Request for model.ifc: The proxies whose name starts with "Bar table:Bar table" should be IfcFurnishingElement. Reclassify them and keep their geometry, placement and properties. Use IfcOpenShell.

First a look at what the model holds.

```python
import re

import ifcopenshell

model = ifcopenshell.open("model.ifc")
print(model.schema)
seen = {}
for e in model.by_type("IfcBuildingElementProxy"):
    name = re.sub(r":\d+(:\d+)?$", "", e.Name or "")  # drop the element id that some exporters append
    seen[name] = seen.get(name, 0) + 1
for name, count in sorted(seen.items()):
    print(count, "x", name)
```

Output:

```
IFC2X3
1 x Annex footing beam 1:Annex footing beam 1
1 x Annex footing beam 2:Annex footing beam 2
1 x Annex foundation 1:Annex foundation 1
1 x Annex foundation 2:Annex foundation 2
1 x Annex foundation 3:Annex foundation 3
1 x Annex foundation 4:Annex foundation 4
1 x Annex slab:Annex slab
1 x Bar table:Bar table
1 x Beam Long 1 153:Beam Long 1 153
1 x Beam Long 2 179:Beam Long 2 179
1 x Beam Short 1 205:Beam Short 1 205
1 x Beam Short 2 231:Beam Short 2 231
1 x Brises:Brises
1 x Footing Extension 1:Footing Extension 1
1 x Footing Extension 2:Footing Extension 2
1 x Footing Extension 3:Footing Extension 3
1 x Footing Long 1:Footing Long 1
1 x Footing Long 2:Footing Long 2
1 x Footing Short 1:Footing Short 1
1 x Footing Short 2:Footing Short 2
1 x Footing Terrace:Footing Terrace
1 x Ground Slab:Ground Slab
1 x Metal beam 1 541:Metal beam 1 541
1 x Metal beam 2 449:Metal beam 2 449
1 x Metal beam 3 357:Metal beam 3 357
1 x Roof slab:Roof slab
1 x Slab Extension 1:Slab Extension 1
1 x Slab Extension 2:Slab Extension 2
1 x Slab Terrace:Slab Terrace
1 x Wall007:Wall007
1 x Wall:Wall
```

```python
import ifcopenshell
import ifcopenshell.api.root

model = ifcopenshell.open("model.ifc")

proxies = [e.id() for e in model.by_type("IfcBuildingElementProxy") if (e.Name or "").startswith("Bar table:Bar table")]
for step_id in proxies:
    proxy = model.by_id(step_id)
    ifcopenshell.api.root.reassign_class(model, product=proxy, ifc_class="IfcFurnishingElement")

print(sum(model.by_id(i).is_a("IfcFurnishingElement") for i in proxies), "reclassified")

model.write("model_v2.ifc")
```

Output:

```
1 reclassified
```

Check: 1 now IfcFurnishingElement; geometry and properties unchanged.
